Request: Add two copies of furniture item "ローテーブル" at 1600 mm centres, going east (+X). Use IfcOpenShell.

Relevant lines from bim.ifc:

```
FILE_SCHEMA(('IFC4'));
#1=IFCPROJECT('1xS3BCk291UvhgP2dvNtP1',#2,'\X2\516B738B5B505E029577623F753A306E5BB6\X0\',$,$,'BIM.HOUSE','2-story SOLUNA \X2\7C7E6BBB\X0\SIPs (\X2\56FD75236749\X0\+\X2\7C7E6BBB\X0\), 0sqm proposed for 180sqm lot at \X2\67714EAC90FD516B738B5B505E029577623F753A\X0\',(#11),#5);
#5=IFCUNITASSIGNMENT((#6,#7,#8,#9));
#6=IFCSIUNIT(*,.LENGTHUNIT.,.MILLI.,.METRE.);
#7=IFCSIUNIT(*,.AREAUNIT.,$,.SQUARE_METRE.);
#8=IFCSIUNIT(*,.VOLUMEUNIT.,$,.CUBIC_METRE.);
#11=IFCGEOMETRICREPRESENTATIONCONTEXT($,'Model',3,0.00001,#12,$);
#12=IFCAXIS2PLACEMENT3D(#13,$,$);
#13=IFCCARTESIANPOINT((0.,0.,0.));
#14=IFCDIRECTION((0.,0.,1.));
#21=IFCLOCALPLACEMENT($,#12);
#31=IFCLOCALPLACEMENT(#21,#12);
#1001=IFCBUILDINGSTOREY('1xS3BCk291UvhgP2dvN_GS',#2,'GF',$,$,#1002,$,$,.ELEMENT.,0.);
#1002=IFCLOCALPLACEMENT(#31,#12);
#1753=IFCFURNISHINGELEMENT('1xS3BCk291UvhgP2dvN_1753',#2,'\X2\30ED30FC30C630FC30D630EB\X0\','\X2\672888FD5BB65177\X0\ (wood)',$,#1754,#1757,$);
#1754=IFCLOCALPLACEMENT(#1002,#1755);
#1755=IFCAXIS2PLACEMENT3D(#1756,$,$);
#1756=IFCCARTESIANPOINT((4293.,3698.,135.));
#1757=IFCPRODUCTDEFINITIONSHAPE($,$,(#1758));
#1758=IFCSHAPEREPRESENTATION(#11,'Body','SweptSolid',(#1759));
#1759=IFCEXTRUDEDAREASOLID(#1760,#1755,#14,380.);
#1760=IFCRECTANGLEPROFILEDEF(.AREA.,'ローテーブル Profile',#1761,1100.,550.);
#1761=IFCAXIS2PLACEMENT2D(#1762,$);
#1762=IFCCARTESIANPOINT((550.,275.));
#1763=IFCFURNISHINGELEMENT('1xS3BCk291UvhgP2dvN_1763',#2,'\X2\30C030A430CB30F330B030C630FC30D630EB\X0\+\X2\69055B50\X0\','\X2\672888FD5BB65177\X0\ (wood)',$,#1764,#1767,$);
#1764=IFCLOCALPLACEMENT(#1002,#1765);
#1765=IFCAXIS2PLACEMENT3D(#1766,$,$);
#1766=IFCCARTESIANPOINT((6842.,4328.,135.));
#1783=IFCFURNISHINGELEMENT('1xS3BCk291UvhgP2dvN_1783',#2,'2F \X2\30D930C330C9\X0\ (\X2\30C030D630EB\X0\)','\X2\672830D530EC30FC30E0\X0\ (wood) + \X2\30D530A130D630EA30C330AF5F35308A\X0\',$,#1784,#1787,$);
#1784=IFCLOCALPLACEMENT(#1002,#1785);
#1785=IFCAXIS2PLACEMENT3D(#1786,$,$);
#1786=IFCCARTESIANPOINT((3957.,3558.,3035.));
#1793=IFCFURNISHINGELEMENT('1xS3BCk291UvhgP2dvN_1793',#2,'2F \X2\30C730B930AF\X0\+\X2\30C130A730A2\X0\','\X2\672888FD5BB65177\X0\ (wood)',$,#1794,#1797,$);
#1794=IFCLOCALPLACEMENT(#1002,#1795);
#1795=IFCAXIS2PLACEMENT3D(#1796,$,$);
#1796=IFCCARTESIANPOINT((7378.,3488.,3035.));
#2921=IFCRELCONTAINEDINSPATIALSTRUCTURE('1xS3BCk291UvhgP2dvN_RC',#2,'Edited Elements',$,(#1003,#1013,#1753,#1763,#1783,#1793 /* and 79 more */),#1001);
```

```python
import numpy as np
import ifcopenshell
import ifcopenshell.api.geometry
import ifcopenshell.api.root
import ifcopenshell.util.element
import ifcopenshell.util.placement

model = ifcopenshell.open("bim.ifc")


def reuse_history(source, copy):
    """copy_class also copies each property set's owner history, people and application; keep the originals."""
    for rel in copy.IsDefinedBy:
        if rel.is_a("IfcRelDefinesByProperties") and (history := rel.RelatingPropertyDefinition.OwnerHistory):
            rel.RelatingPropertyDefinition.OwnerHistory = source.OwnerHistory
            ifcopenshell.util.element.remove_deep2(model, history)


source = model.by_guid("1xS3BCk291UvhgP2dvN_1753")
base = ifcopenshell.util.placement.get_local_placement(source.ObjectPlacement)
step = np.array([1.0, 0.0, 0.0]) * 1600.0

for i in range(1, 3):
    copy = ifcopenshell.api.root.copy_class(model, product=source)
    copy.Representation = ifcopenshell.util.element.copy_deep(
        model, source.Representation, exclude=["IfcGeometricRepresentationContext", "IfcRepresentationMap"]
    )
    reuse_history(source, copy)
    matrix = base.copy()
    matrix[:3, 3] += i * step
    print("added at", matrix[:3, 3].round(3) + 0.0)
    ifcopenshell.api.geometry.edit_object_placement(model, product=copy, matrix=matrix, is_si=False)

model.write("bim_rev.ifc")
```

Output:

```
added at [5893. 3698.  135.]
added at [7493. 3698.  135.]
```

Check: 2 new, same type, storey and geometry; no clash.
